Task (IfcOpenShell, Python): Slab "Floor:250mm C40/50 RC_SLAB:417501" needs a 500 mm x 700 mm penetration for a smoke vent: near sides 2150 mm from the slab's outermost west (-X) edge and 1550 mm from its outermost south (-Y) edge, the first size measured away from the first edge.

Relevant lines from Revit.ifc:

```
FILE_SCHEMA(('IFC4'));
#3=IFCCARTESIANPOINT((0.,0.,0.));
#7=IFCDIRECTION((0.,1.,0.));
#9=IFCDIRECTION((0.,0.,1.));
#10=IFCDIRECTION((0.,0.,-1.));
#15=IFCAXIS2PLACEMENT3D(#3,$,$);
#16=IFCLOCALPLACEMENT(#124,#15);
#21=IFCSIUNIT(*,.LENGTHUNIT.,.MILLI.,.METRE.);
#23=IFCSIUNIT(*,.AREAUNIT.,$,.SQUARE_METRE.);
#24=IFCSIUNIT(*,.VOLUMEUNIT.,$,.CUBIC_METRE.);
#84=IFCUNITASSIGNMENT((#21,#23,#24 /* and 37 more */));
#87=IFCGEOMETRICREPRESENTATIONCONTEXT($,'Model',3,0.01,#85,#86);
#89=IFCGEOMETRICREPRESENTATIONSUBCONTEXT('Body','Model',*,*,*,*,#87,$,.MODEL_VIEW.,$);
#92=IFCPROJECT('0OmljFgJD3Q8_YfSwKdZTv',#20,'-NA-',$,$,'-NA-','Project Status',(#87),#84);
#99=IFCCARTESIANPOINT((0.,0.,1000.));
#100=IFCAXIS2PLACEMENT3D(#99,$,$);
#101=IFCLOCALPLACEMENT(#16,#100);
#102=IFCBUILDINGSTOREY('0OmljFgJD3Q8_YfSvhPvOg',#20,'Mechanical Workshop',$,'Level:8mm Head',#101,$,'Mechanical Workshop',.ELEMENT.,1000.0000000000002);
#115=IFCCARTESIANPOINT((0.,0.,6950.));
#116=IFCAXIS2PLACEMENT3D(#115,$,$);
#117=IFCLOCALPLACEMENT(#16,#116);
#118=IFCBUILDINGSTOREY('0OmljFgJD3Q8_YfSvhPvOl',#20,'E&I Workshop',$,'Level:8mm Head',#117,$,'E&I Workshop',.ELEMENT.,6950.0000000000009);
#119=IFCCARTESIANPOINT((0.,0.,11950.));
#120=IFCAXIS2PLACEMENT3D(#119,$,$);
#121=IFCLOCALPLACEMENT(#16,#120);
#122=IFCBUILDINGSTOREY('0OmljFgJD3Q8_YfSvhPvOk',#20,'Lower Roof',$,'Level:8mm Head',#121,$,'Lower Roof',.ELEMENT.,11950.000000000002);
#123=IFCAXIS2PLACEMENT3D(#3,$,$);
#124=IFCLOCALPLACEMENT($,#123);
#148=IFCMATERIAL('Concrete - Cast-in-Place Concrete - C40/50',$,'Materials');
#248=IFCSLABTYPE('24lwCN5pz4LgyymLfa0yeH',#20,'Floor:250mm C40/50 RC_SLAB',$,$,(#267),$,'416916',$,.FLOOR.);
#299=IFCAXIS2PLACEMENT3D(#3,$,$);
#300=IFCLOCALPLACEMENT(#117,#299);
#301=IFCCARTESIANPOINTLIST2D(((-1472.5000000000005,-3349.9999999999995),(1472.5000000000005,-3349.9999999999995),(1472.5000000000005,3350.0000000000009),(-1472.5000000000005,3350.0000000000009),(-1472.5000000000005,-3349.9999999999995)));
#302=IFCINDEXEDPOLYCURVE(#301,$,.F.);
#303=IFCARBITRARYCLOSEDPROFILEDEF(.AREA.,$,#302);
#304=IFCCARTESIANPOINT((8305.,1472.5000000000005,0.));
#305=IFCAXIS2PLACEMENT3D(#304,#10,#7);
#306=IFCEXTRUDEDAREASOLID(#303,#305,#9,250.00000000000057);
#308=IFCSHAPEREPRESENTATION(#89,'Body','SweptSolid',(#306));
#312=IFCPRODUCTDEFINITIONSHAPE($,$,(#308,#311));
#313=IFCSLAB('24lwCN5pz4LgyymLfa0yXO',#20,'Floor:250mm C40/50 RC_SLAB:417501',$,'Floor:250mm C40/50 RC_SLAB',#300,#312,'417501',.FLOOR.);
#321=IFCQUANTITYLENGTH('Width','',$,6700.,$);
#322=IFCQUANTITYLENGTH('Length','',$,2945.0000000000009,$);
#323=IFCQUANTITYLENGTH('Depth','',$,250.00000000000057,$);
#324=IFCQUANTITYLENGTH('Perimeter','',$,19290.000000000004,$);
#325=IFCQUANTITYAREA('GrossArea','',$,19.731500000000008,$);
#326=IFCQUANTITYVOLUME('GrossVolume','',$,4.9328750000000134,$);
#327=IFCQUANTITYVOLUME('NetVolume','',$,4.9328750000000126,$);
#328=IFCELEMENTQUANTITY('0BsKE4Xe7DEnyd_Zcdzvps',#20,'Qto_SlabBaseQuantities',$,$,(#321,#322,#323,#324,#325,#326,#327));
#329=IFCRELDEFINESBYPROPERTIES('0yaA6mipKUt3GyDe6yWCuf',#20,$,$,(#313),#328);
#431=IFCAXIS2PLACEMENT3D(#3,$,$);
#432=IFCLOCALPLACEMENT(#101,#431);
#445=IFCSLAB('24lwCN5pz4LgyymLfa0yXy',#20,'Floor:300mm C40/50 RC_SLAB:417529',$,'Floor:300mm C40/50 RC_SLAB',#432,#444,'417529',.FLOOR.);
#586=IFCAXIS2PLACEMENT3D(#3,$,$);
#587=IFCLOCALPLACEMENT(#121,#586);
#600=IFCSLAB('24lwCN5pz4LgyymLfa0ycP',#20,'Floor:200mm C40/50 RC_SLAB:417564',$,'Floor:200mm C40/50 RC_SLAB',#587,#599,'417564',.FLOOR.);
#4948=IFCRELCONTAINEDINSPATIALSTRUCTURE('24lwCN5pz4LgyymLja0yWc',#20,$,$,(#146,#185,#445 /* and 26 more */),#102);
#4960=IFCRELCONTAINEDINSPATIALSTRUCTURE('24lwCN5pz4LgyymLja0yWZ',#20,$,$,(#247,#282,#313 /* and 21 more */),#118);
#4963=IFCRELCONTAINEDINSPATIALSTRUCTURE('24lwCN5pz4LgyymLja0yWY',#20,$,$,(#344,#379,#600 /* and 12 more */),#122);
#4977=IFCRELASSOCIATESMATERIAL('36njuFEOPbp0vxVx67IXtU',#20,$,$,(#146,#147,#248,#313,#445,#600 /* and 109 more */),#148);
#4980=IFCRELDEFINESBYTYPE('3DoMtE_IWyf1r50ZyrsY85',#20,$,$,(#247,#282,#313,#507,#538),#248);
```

```python
import numpy as np
import ifcopenshell
import ifcopenshell.api.feature
import ifcopenshell.api.geometry
import ifcopenshell.api.pset
import ifcopenshell.api.root
import ifcopenshell.geom
import ifcopenshell.util.element
import ifcopenshell.util.placement
import ifcopenshell.util.representation
import ifcopenshell.util.shape
import ifcopenshell.util.unit

model = ifcopenshell.open("Revit.ifc")
unit_scale = ifcopenshell.util.unit.calculate_unit_scale(model)
volume_scale = ifcopenshell.util.unit.calculate_unit_scale(model, "VOLUMEUNIT")
settings = ifcopenshell.geom.settings()


def volume(element):
    """Net volume in cubic metres, openings subtracted."""
    shape = ifcopenshell.geom.create_shape(settings, element)
    return ifcopenshell.util.shape.get_volume(shape.geometry)


slab = model.by_guid("24lwCN5pz4LgyymLfa0yXO")
before = volume(slab)

# Extent in the slab's own axes, in metres. The edges named are its -X and -Y sides.
slab_shape = ifcopenshell.geom.create_shape(settings, slab)
vertices = ifcopenshell.util.shape.get_vertices(slab_shape.geometry)
x_min, y_min, bottom = vertices.min(axis=0)
top = vertices[:, 2].max()

opening = ifcopenshell.api.root.create_entity(model, ifc_class="IfcOpeningElement", name="Smoke vent opening", predefined_type="OPENING")
context = ifcopenshell.util.representation.get_context(model, "Model", "Body", "MODEL_VIEW")
width, depth = 0.5, 0.7
outline = [(0.0, 0.0), (width, 0.0), (width, depth), (0.0, depth), (0.0, 0.0)]
# Overshoot both faces by 50 mm so the cut is clean.
shape = ifcopenshell.api.geometry.add_slab_representation(
    model, context=context, depth=top - bottom + 0.1, polyline=outline
)
ifcopenshell.api.geometry.assign_representation(model, product=opening, representation=shape)

matrix = ifcopenshell.util.placement.get_local_placement(slab.ObjectPlacement)
matrix[:, 3] = matrix @ np.append(np.array([x_min + 2.15, y_min + 1.55, bottom - 0.05]) / unit_scale, 1.0)
ifcopenshell.api.geometry.edit_object_placement(model, product=opening, matrix=matrix, is_si=False)
ifcopenshell.api.feature.add_feature(model, feature=opening, element=slab)

after = volume(slab)

# Update the slab's stored quantities.
qto = model.by_id(ifcopenshell.util.element.get_pset(slab, "Qto_SlabBaseQuantities", should_inherit=False)["id"])
ifcopenshell.api.pset.edit_qto(model, qto=qto, properties={"NetVolume": after / volume_scale})

print(f"slab volume {before:.3f} -> {after:.3f} m3")

model.write("Revit-out.ifc")
```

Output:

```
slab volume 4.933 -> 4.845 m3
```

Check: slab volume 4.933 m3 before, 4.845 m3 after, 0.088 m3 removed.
